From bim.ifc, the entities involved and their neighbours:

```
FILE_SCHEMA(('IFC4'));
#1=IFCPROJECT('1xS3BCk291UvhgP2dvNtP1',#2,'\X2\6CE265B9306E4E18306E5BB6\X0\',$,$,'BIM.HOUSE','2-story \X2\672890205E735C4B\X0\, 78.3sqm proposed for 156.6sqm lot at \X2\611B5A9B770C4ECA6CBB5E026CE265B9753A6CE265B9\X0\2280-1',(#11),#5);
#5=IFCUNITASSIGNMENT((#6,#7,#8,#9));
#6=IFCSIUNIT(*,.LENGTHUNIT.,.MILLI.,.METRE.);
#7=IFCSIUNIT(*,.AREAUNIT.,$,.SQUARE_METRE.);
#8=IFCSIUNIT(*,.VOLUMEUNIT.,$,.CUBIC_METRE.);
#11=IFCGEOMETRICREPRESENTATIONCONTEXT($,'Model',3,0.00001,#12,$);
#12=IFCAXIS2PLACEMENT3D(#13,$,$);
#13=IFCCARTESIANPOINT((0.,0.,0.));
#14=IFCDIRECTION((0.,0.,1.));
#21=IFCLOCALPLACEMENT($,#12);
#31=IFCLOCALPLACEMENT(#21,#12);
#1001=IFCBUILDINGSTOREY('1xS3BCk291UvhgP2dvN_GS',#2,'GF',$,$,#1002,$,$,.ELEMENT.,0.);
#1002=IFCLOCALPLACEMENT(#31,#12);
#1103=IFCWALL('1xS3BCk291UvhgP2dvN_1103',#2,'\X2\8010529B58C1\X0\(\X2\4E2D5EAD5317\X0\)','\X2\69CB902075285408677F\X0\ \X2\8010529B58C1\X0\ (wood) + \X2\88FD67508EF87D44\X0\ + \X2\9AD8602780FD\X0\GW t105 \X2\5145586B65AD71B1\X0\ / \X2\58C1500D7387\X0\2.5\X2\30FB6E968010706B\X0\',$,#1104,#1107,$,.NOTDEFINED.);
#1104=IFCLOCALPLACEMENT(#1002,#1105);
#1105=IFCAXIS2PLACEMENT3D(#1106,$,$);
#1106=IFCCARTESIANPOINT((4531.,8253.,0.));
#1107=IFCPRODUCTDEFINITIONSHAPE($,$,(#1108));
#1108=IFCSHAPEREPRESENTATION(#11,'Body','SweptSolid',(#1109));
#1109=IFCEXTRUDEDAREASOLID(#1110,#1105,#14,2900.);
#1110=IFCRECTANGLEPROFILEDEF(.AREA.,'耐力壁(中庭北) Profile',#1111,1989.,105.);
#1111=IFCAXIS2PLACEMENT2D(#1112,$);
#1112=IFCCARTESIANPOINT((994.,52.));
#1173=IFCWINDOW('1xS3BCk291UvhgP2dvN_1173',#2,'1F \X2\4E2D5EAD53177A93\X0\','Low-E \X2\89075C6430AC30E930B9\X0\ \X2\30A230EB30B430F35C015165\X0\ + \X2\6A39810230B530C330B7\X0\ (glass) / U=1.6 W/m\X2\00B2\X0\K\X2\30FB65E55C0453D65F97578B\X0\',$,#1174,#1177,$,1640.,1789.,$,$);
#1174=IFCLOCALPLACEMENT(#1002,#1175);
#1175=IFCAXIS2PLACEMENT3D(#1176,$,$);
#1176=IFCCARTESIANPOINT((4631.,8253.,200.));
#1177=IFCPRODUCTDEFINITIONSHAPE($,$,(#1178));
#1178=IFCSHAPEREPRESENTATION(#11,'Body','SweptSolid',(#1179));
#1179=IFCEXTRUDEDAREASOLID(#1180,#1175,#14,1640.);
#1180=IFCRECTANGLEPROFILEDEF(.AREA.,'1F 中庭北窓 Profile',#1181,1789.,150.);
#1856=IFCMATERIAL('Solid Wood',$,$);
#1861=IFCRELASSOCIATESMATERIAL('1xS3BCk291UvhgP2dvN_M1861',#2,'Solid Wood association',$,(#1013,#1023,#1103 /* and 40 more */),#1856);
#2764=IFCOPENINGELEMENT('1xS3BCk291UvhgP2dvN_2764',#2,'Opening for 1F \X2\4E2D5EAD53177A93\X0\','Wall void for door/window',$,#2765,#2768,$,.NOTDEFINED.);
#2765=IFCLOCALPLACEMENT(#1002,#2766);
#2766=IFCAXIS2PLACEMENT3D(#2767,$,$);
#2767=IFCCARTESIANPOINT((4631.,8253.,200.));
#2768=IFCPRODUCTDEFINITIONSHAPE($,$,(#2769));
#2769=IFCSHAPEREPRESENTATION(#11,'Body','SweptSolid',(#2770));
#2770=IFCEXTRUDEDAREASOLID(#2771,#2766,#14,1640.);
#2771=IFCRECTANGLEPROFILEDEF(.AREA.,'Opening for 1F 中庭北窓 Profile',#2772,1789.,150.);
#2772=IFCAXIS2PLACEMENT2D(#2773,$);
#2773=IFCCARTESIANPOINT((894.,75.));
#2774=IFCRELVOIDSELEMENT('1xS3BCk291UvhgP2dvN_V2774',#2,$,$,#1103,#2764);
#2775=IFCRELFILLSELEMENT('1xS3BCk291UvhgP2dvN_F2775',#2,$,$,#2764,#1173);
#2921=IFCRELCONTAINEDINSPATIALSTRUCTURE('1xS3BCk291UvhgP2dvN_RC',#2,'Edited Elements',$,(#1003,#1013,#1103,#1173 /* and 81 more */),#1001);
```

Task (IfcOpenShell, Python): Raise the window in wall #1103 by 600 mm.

```python
import numpy as np
import ifcopenshell
import ifcopenshell.api.geometry
import ifcopenshell.util.placement
import ifcopenshell.util.unit

model = ifcopenshell.open("bim.ifc")
unit_scale = ifcopenshell.util.unit.calculate_unit_scale(model)

window = model.by_guid("1xS3BCk291UvhgP2dvN_1173")
opening = window.FillsVoids[0].RelatingOpeningElement
dz = 0.6 / unit_scale

shift = np.array([0.0, 0.0, dz])
# The window is not placed relative to its opening, so move both.
for product in (opening, window):
    matrix = ifcopenshell.util.placement.get_local_placement(product.ObjectPlacement)
    matrix[:3, 3] += shift
    ifcopenshell.api.geometry.edit_object_placement(model, product=product, matrix=matrix, is_si=False)

print(f"moved by {dz * unit_scale:+.3f} m")

model.write("bim_rev.ifc")
```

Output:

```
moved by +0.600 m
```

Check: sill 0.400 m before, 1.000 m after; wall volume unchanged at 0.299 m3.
